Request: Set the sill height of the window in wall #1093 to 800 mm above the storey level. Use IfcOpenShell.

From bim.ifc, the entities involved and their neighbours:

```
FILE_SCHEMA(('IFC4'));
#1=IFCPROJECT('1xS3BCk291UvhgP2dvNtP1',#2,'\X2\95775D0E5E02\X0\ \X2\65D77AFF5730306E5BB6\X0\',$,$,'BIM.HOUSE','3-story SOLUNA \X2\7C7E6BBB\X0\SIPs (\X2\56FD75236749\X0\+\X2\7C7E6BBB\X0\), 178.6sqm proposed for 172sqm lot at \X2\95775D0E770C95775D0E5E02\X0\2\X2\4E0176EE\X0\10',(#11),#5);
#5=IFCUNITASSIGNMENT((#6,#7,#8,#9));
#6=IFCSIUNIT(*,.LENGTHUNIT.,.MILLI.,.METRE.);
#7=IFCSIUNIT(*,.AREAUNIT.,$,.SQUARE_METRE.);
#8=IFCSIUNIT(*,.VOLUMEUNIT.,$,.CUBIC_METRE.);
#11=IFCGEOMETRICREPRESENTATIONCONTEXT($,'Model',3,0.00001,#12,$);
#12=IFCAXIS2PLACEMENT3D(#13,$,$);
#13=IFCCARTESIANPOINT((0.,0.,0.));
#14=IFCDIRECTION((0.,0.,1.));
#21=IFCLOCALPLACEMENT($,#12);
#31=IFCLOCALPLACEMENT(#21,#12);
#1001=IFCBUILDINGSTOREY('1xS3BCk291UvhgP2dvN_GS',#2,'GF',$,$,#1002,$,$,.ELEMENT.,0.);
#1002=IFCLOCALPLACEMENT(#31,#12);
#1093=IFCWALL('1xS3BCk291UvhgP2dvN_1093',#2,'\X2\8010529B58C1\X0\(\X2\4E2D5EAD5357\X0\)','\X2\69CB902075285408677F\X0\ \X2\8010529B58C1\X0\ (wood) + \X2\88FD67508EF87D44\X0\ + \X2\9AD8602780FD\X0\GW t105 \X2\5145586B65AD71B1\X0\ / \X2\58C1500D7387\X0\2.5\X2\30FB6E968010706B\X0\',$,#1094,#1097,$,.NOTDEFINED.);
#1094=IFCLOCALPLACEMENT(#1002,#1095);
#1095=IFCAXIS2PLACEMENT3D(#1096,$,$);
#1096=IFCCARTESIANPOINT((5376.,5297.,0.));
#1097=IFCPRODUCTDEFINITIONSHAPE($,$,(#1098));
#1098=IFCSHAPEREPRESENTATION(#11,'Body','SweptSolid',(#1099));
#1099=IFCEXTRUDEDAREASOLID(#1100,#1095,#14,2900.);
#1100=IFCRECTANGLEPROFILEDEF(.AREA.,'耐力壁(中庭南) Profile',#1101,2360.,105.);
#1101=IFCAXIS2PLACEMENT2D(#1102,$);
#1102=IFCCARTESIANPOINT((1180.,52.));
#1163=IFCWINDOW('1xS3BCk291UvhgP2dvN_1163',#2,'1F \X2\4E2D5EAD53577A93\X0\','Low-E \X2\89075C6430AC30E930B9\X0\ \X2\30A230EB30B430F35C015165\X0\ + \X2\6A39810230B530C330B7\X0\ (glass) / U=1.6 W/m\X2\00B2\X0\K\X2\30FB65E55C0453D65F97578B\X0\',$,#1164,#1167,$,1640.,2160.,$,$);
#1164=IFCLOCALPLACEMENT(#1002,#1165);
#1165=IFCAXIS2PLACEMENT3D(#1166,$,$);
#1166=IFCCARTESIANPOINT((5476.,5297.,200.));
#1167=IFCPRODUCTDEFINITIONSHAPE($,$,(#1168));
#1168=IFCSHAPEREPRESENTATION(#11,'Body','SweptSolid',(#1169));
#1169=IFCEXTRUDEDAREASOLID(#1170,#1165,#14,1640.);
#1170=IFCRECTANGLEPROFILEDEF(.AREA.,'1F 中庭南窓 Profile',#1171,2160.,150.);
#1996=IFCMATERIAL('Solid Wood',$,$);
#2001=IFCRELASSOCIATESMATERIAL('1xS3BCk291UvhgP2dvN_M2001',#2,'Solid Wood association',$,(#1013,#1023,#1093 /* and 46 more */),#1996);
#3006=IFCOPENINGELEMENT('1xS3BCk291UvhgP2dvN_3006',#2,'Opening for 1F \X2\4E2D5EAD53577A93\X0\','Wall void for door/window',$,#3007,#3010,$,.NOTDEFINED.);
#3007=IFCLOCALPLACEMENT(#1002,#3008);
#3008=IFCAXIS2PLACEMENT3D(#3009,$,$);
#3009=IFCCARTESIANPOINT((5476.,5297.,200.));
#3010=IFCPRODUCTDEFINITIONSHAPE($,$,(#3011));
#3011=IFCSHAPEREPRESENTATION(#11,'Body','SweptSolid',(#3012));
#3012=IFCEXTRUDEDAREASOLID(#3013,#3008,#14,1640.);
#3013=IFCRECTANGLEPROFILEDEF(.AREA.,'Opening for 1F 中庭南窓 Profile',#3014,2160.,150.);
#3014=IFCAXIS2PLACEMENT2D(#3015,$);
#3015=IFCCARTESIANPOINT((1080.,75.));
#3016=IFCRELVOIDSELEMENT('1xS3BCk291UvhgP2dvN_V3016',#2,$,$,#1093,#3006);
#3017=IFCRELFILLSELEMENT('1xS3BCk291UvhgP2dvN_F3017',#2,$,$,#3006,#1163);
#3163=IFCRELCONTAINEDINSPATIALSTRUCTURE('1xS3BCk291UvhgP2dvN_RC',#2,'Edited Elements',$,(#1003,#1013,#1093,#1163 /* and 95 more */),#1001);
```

```python
import numpy as np
import ifcopenshell
import ifcopenshell.api.geometry
import ifcopenshell.geom
import ifcopenshell.util.element
import ifcopenshell.util.placement
import ifcopenshell.util.shape
import ifcopenshell.util.unit

model = ifcopenshell.open("bim.ifc")
unit_scale = ifcopenshell.util.unit.calculate_unit_scale(model)

window = model.by_guid("1xS3BCk291UvhgP2dvN_1163")
opening = window.FillsVoids[0].RelatingOpeningElement
storey = ifcopenshell.util.element.get_container(window, ifc_class="IfcBuildingStorey")
level = ifcopenshell.util.placement.get_local_placement(storey.ObjectPlacement)[2, 3]

# The opening's origin need not be at the sill, so measure its lowest point.
shape = ifcopenshell.geom.create_shape(ifcopenshell.geom.settings(), opening)
bottom = ifcopenshell.util.shape.get_shape_bottom_elevation(shape, shape.geometry) / unit_scale
dz = level + 800.0 - bottom

shift = np.array([0.0, 0.0, dz])
# The window is not placed relative to its opening, so move both.
for product in (opening, window):
    matrix = ifcopenshell.util.placement.get_local_placement(product.ObjectPlacement)
    matrix[:3, 3] += shift
    ifcopenshell.api.geometry.edit_object_placement(model, product=product, matrix=matrix, is_si=False)

print(f"moved by {dz * unit_scale:+.3f} m")

model.write("bim_updated.ifc")
```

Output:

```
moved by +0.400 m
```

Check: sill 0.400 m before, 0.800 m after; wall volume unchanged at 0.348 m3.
